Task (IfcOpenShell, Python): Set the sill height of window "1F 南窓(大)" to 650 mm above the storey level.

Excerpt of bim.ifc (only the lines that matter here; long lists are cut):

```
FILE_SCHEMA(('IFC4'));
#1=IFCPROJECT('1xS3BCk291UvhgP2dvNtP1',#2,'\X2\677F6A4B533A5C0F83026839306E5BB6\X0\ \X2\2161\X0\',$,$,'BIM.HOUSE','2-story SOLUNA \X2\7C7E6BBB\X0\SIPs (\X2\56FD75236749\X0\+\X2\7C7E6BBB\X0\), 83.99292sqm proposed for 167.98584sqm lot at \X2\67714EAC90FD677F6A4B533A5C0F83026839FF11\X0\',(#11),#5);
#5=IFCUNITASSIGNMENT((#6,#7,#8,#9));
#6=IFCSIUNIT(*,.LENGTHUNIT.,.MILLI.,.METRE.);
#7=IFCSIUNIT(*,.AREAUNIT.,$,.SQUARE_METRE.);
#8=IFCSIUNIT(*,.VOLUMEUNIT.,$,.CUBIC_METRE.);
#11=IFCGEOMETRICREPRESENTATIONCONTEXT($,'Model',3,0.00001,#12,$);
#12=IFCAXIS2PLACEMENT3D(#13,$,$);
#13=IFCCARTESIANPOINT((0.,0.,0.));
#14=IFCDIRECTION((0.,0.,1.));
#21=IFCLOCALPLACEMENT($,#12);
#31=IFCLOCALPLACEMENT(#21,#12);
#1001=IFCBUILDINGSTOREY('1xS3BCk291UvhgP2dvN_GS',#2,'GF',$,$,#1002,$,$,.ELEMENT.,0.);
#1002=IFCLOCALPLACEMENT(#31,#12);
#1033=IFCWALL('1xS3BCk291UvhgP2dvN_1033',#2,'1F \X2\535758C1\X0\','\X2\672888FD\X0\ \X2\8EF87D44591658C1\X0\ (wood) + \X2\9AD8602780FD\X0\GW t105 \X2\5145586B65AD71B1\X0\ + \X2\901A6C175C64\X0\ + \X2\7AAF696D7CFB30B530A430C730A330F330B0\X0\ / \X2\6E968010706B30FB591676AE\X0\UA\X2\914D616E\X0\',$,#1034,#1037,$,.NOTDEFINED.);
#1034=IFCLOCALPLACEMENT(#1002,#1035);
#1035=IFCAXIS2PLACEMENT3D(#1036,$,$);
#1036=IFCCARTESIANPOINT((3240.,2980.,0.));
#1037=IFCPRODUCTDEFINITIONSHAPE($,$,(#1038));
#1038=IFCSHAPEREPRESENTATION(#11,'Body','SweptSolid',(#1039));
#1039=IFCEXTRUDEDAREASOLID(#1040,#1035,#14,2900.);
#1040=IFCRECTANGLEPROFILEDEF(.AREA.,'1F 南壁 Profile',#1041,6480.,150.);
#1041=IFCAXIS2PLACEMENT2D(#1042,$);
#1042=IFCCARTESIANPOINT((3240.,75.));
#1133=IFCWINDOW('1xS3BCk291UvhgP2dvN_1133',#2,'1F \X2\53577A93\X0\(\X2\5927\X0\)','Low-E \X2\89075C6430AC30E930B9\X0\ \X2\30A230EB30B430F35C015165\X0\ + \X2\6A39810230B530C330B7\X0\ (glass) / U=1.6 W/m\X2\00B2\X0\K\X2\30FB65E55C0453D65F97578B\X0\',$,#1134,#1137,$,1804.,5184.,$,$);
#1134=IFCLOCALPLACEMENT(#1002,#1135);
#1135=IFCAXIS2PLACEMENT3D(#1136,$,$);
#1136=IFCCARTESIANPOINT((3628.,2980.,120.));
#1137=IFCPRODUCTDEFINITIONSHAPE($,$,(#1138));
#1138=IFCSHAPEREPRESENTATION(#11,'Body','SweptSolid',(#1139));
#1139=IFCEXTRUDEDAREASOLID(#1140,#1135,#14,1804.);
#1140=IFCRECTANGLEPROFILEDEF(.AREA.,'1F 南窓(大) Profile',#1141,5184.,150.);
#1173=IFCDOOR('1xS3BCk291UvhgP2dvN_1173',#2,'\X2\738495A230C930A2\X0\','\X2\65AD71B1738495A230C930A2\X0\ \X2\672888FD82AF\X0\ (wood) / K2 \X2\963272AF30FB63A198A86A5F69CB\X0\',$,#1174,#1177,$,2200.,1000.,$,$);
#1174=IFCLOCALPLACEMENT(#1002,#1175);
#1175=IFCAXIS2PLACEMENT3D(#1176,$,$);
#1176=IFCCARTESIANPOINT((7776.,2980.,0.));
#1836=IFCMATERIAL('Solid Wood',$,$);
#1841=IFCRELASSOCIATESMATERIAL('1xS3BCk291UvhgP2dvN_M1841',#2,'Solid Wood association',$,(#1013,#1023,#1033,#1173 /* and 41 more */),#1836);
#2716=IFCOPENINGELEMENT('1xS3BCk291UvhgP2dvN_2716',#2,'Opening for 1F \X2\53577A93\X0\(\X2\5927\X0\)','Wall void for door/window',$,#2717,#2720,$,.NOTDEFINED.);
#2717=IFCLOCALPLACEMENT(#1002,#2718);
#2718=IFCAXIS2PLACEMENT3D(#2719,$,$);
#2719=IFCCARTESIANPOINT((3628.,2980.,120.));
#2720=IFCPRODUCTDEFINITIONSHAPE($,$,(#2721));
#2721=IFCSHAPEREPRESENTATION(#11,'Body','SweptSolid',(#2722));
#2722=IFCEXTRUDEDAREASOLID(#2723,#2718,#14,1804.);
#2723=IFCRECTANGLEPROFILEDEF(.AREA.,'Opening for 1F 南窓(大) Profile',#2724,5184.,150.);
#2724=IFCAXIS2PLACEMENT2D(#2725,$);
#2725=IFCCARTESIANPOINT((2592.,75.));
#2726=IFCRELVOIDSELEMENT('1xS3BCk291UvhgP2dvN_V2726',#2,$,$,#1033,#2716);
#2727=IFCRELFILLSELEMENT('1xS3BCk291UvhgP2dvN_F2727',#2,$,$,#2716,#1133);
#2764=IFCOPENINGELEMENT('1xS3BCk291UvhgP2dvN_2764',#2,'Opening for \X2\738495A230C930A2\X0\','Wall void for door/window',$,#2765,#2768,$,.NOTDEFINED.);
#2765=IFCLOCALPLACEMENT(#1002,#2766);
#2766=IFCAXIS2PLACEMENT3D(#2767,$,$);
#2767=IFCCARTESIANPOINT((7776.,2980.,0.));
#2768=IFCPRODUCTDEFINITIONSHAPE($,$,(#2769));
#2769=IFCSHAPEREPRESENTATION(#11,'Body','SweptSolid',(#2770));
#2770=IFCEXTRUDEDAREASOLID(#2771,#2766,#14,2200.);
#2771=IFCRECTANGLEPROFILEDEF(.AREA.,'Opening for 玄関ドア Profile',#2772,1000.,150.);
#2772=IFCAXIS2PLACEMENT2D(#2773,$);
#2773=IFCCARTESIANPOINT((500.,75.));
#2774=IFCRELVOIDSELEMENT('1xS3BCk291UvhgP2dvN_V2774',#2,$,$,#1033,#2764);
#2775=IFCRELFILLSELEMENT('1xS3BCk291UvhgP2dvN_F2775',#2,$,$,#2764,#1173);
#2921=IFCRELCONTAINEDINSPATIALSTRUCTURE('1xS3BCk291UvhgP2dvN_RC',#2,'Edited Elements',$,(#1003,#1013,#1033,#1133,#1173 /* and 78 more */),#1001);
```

```python
import numpy as np
import ifcopenshell
import ifcopenshell.api.geometry
import ifcopenshell.geom
import ifcopenshell.util.element
import ifcopenshell.util.placement
import ifcopenshell.util.shape
import ifcopenshell.util.unit

model = ifcopenshell.open("bim.ifc")
unit_scale = ifcopenshell.util.unit.calculate_unit_scale(model)

window = model.by_guid("1xS3BCk291UvhgP2dvN_1133")
opening = window.FillsVoids[0].RelatingOpeningElement
storey = ifcopenshell.util.element.get_container(window, ifc_class="IfcBuildingStorey")
level = ifcopenshell.util.placement.get_local_placement(storey.ObjectPlacement)[2, 3]

# The opening's origin need not be at the sill, so measure its lowest point.
shape = ifcopenshell.geom.create_shape(ifcopenshell.geom.settings(), opening)
bottom = ifcopenshell.util.shape.get_shape_bottom_elevation(shape, shape.geometry) / unit_scale
dz = level + 650.0 - bottom

shift = np.array([0.0, 0.0, dz])
# The window is not placed relative to its opening, so move both.
for product in (opening, window):
    matrix = ifcopenshell.util.placement.get_local_placement(product.ObjectPlacement)
    matrix[:3, 3] += shift
    ifcopenshell.api.geometry.edit_object_placement(model, product=product, matrix=matrix, is_si=False)

print(f"moved by {dz * unit_scale:+.3f} m")

model.write("bim_edited.ifc")
```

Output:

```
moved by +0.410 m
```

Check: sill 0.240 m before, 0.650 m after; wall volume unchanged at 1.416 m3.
